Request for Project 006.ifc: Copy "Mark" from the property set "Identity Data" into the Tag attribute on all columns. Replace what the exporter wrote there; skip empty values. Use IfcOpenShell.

First a look at what the model holds.

```python
import ifcopenshell
import ifcopenshell.util.element

model = ifcopenshell.open("Project 006.ifc")
print(model.schema)
columns = model.by_type("IfcColumn")
print(len(columns), "columns")
for e in columns[:8]:
    source = ifcopenshell.util.element.get_pset(e, "Identity Data", "Mark")
    target = e.Tag
    print(e.id(), repr(source), repr(target), sep=" | ")
```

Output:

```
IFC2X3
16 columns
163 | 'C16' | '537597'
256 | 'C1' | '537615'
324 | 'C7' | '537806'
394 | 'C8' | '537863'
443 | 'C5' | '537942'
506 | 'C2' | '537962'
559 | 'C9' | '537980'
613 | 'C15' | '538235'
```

```python
import ifcopenshell
import ifcopenshell.util.element

model = ifcopenshell.open("Project 006.ifc")

count = 0
for e in model.by_type("IfcColumn"):
    value = ifcopenshell.util.element.get_pset(e, "Identity Data", "Mark")
    current = e.Tag
    if not value or not value.strip() or current == value:
        continue
    e.Tag = value
    count += 1

print(count, "columns updated")

model.write("Project 006_edited.ifc")
```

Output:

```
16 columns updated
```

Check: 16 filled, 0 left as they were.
